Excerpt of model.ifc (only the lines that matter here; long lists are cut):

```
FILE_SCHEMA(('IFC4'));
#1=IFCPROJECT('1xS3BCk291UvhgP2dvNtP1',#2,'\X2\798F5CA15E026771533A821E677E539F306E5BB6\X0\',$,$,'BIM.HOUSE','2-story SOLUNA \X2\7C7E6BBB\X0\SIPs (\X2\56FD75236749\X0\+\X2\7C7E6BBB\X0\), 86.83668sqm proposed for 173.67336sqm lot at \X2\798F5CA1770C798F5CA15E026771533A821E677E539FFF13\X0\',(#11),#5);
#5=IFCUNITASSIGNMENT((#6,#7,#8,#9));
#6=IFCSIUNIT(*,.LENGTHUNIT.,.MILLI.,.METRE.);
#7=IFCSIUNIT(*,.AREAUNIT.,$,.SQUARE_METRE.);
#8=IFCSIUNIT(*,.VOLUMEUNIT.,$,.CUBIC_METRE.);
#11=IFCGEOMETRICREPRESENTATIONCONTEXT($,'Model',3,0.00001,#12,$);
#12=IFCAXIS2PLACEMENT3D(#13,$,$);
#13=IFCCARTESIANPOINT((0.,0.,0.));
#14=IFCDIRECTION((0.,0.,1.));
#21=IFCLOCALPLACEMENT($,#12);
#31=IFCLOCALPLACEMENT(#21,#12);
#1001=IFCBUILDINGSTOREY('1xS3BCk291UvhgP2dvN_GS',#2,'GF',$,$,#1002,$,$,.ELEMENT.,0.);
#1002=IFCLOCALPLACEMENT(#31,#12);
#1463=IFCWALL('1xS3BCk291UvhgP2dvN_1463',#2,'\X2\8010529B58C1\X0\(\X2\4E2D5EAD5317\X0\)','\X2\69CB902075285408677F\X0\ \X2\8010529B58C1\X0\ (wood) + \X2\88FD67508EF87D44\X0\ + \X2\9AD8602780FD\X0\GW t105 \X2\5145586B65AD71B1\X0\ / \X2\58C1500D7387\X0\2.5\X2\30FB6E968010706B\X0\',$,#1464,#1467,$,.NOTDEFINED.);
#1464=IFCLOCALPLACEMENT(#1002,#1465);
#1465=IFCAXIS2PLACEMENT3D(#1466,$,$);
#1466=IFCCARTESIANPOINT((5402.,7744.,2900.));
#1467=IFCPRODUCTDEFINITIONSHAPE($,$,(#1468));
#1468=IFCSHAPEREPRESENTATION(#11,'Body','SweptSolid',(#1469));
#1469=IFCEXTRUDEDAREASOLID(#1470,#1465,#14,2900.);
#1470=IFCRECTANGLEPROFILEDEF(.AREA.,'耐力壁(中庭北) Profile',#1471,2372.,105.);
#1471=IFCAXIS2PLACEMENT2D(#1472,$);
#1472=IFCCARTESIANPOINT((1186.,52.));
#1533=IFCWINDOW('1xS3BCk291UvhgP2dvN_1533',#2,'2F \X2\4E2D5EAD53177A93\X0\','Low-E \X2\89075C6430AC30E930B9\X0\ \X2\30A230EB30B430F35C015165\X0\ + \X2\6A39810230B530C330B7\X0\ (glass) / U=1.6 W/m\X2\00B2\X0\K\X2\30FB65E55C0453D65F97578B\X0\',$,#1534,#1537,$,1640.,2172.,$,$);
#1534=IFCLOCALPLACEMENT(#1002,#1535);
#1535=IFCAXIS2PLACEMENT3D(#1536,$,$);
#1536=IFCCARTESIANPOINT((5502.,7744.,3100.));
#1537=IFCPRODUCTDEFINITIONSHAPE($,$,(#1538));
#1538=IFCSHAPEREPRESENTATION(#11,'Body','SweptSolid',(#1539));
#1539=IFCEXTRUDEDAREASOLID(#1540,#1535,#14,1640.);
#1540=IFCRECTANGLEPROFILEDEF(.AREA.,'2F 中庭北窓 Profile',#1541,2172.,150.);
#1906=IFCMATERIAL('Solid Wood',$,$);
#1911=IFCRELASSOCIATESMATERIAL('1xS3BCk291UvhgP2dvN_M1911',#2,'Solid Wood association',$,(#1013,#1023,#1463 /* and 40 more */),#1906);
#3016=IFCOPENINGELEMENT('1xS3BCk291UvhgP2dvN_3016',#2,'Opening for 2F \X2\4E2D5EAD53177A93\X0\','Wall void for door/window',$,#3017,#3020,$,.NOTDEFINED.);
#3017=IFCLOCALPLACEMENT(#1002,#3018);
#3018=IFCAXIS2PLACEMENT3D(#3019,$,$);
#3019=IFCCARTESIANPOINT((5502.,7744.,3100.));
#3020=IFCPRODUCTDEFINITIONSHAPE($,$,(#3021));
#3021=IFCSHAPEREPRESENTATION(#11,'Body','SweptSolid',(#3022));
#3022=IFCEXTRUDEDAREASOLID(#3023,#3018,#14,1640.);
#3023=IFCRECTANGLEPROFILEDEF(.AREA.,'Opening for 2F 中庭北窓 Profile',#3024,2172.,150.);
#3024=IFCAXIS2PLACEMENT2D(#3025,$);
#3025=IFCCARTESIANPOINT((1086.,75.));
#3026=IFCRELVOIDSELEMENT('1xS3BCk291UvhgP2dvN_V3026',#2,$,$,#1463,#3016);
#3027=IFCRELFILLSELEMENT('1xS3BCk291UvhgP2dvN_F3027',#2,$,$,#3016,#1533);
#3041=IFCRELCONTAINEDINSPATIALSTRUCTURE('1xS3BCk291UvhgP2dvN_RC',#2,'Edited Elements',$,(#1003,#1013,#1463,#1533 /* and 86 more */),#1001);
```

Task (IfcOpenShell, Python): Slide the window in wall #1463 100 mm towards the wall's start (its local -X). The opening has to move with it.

```python
import ifcopenshell
import ifcopenshell.api.geometry
import ifcopenshell.util.placement

model = ifcopenshell.open("model.ifc")

window = model.by_guid("1xS3BCk291UvhgP2dvN_1533")
opening = window.FillsVoids[0].RelatingOpeningElement
wall = opening.VoidsElements[0].RelatingBuildingElement

wall_matrix = ifcopenshell.util.placement.get_local_placement(wall.ObjectPlacement)
shift = wall_matrix[:3, 0] * -100.0
before = ifcopenshell.util.placement.get_local_placement(window.ObjectPlacement)[:3, 3].copy()

# The window is not placed relative to its opening, so move both.
for product in (opening, window):
    matrix = ifcopenshell.util.placement.get_local_placement(product.ObjectPlacement)
    matrix[:3, 3] += shift
    ifcopenshell.api.geometry.edit_object_placement(model, product=product, matrix=matrix, is_si=False)

after = ifcopenshell.util.placement.get_local_placement(window.ObjectPlacement)[:3, 3]
print("window moved by", (after - before).round(3) + 0.0)

model.write("model_edited.ifc")
```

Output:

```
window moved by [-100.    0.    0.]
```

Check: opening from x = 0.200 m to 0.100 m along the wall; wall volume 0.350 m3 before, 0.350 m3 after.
